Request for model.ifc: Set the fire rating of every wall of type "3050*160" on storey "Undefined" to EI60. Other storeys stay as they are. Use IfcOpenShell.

First a look at what the model holds.

```python
import ifcopenshell
import ifcopenshell.util.element

model = ifcopenshell.open("model.ifc")
print(model.schema)
storey = next(s for s in model.by_type("IfcBuildingStorey") if s.Name == "Undefined")
walls = [e for e in ifcopenshell.util.element.get_decomposition(storey) if e.is_a("IfcWall")]
seen = {}
for e in walls:
    element_type = ifcopenshell.util.element.get_type(e)
    key = (element_type.Name if element_type != e and element_type else None, ifcopenshell.util.element.get_pset(e, "Pset_WallCommon", "FireRating"))
    seen[key] = seen.get(key, 0) + 1
for (name, value), count in sorted(seen.items(), key=str):
    print(count, "x", name, "|", value)
```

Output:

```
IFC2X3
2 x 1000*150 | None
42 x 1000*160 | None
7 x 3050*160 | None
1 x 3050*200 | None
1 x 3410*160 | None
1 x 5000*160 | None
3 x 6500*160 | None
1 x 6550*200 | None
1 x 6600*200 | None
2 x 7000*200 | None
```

```python
import ifcopenshell
import ifcopenshell.api.pset
import ifcopenshell.util.element

model = ifcopenshell.open("model.ifc")

storey = next(s for s in model.by_type("IfcBuildingStorey") if s.Name == "Undefined")
walls = [e for e in ifcopenshell.util.element.get_decomposition(storey) if e.is_a("IfcWall")]

count = 0
for e in walls:
    element_type = ifcopenshell.util.element.get_type(e)
    if element_type in (None, e) or element_type.Name != "3050*160":
        continue
    # add_pset returns the element's existing set when there is one.
    pset = ifcopenshell.api.pset.add_pset(model, product=e, name="Pset_WallCommon")
    ifcopenshell.api.pset.edit_pset(model, pset=pset, properties={"FireRating": "EI60"})
    count += 1

print(count, "walls updated")

model.write("model_v2.ifc")
```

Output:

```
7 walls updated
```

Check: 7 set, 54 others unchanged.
